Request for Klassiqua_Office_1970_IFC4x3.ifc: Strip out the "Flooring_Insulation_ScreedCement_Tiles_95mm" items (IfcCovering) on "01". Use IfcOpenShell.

First a look at what the model holds.

```python
import ifcopenshell
import ifcopenshell.util.element

model = ifcopenshell.open("Klassiqua_Office_1970_IFC4x3.ifc")
print(model.schema)
storey = next(s for s in model.by_type("IfcBuildingStorey") if s.Name == "01")
coverings = [e for e in ifcopenshell.util.element.get_decomposition(storey) if e.is_a("IfcCovering")]
seen = {}
for e in coverings:
    element_type = ifcopenshell.util.element.get_type(e)
    name = element_type.Name if element_type not in (None, e) else None
    seen[name] = seen.get(name, 0) + 1
for name, count in sorted(seen.items(), key=str):
    print(count, "x", name)
```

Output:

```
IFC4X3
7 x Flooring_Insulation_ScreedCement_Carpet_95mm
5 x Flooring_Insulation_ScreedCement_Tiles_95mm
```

```python
import ifcopenshell
import ifcopenshell.api.root
import ifcopenshell.util.element

model = ifcopenshell.open("Klassiqua_Office_1970_IFC4x3.ifc")

storey = next(s for s in model.by_type("IfcBuildingStorey") if s.Name == "01")
coverings = [e for e in ifcopenshell.util.element.get_decomposition(storey) if e.is_a("IfcCovering")]
targets = [e for e in coverings if (t := ifcopenshell.util.element.get_type(e)) not in (None, e) and t.Name == "Flooring_Insulation_ScreedCement_Tiles_95mm"]

for e in targets:
    ifcopenshell.api.root.remove_product(model, product=e)
print(len(targets), "removed")

model.write("Klassiqua_Office_1970_IFC4x3_edited.ifc")
```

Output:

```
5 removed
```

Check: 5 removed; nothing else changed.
